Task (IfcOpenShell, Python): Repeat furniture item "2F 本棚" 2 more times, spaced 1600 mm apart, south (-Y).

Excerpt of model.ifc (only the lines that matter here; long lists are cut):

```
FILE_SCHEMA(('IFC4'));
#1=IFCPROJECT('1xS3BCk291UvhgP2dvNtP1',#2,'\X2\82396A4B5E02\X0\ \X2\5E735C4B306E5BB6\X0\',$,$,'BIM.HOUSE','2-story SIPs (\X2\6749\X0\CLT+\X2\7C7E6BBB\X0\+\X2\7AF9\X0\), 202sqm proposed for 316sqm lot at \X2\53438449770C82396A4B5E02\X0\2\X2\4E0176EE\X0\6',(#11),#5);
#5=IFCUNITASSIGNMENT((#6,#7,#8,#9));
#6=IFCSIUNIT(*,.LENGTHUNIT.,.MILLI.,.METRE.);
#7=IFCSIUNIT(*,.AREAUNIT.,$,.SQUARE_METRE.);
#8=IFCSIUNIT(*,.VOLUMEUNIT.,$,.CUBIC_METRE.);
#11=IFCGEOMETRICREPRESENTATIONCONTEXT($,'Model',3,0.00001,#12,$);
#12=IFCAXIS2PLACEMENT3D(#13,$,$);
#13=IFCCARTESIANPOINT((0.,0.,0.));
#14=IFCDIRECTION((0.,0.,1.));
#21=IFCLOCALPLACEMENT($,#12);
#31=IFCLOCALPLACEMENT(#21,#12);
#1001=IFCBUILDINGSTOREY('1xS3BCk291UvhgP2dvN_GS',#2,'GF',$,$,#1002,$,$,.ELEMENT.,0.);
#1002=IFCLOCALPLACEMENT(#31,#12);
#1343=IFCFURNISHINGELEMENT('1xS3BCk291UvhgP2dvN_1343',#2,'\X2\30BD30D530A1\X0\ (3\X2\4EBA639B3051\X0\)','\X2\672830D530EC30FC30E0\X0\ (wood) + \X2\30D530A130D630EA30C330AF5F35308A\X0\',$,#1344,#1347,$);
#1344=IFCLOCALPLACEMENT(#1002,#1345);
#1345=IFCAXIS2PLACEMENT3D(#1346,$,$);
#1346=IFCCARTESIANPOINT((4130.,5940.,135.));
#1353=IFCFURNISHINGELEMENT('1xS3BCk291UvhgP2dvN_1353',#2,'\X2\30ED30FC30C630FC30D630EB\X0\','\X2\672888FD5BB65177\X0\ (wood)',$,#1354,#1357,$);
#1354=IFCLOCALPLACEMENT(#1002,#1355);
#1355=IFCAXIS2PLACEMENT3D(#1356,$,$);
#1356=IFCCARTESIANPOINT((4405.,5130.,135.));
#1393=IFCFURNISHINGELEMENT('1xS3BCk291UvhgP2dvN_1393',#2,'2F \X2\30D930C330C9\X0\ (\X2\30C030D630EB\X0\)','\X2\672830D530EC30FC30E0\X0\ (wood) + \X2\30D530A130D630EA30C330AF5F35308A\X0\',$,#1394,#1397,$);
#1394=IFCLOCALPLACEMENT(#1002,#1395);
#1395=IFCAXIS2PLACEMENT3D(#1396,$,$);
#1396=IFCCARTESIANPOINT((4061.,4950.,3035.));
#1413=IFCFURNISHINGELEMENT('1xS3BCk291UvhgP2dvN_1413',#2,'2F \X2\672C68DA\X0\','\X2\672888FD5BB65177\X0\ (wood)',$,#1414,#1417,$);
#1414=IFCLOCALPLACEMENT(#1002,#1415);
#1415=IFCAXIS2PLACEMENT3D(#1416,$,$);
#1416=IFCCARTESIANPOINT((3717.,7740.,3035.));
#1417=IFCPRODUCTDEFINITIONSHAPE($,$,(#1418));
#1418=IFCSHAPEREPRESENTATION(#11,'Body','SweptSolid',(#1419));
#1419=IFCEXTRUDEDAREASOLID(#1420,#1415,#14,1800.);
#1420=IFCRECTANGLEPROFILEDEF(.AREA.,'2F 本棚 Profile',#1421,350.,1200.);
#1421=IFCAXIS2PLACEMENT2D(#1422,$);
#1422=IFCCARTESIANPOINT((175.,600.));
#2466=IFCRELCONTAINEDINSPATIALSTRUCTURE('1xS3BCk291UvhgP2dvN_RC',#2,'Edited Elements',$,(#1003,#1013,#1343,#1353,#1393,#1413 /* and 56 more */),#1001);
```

```python
import numpy as np
import ifcopenshell
import ifcopenshell.api.geometry
import ifcopenshell.api.root
import ifcopenshell.util.element
import ifcopenshell.util.placement
import ifcopenshell.util.unit

model = ifcopenshell.open("model.ifc")
unit_scale = ifcopenshell.util.unit.calculate_unit_scale(model)


def reuse_history(source, copy):
    """copy_class also copies each property set's owner history, people and application; keep the originals."""
    for rel in copy.IsDefinedBy:
        if rel.is_a("IfcRelDefinesByProperties") and (history := rel.RelatingPropertyDefinition.OwnerHistory):
            rel.RelatingPropertyDefinition.OwnerHistory = source.OwnerHistory
            ifcopenshell.util.element.remove_deep2(model, history)


source = model.by_id(1413)
base = ifcopenshell.util.placement.get_local_placement(source.ObjectPlacement)
step = np.array([0.0, -1.0, 0.0]) * 1.6 / unit_scale

for i in range(1, 3):
    copy = ifcopenshell.api.root.copy_class(model, product=source)
    copy.Representation = ifcopenshell.util.element.copy_deep(
        model, source.Representation, exclude=["IfcGeometricRepresentationContext", "IfcRepresentationMap"]
    )
    reuse_history(source, copy)
    matrix = base.copy()
    matrix[:3, 3] += i * step
    print("added at", matrix[:3, 3].round(3) + 0.0)
    ifcopenshell.api.geometry.edit_object_placement(model, product=copy, matrix=matrix, is_si=False)

model.write("model_edited.ifc")
```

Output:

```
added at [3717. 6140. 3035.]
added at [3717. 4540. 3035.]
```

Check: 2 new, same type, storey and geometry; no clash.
